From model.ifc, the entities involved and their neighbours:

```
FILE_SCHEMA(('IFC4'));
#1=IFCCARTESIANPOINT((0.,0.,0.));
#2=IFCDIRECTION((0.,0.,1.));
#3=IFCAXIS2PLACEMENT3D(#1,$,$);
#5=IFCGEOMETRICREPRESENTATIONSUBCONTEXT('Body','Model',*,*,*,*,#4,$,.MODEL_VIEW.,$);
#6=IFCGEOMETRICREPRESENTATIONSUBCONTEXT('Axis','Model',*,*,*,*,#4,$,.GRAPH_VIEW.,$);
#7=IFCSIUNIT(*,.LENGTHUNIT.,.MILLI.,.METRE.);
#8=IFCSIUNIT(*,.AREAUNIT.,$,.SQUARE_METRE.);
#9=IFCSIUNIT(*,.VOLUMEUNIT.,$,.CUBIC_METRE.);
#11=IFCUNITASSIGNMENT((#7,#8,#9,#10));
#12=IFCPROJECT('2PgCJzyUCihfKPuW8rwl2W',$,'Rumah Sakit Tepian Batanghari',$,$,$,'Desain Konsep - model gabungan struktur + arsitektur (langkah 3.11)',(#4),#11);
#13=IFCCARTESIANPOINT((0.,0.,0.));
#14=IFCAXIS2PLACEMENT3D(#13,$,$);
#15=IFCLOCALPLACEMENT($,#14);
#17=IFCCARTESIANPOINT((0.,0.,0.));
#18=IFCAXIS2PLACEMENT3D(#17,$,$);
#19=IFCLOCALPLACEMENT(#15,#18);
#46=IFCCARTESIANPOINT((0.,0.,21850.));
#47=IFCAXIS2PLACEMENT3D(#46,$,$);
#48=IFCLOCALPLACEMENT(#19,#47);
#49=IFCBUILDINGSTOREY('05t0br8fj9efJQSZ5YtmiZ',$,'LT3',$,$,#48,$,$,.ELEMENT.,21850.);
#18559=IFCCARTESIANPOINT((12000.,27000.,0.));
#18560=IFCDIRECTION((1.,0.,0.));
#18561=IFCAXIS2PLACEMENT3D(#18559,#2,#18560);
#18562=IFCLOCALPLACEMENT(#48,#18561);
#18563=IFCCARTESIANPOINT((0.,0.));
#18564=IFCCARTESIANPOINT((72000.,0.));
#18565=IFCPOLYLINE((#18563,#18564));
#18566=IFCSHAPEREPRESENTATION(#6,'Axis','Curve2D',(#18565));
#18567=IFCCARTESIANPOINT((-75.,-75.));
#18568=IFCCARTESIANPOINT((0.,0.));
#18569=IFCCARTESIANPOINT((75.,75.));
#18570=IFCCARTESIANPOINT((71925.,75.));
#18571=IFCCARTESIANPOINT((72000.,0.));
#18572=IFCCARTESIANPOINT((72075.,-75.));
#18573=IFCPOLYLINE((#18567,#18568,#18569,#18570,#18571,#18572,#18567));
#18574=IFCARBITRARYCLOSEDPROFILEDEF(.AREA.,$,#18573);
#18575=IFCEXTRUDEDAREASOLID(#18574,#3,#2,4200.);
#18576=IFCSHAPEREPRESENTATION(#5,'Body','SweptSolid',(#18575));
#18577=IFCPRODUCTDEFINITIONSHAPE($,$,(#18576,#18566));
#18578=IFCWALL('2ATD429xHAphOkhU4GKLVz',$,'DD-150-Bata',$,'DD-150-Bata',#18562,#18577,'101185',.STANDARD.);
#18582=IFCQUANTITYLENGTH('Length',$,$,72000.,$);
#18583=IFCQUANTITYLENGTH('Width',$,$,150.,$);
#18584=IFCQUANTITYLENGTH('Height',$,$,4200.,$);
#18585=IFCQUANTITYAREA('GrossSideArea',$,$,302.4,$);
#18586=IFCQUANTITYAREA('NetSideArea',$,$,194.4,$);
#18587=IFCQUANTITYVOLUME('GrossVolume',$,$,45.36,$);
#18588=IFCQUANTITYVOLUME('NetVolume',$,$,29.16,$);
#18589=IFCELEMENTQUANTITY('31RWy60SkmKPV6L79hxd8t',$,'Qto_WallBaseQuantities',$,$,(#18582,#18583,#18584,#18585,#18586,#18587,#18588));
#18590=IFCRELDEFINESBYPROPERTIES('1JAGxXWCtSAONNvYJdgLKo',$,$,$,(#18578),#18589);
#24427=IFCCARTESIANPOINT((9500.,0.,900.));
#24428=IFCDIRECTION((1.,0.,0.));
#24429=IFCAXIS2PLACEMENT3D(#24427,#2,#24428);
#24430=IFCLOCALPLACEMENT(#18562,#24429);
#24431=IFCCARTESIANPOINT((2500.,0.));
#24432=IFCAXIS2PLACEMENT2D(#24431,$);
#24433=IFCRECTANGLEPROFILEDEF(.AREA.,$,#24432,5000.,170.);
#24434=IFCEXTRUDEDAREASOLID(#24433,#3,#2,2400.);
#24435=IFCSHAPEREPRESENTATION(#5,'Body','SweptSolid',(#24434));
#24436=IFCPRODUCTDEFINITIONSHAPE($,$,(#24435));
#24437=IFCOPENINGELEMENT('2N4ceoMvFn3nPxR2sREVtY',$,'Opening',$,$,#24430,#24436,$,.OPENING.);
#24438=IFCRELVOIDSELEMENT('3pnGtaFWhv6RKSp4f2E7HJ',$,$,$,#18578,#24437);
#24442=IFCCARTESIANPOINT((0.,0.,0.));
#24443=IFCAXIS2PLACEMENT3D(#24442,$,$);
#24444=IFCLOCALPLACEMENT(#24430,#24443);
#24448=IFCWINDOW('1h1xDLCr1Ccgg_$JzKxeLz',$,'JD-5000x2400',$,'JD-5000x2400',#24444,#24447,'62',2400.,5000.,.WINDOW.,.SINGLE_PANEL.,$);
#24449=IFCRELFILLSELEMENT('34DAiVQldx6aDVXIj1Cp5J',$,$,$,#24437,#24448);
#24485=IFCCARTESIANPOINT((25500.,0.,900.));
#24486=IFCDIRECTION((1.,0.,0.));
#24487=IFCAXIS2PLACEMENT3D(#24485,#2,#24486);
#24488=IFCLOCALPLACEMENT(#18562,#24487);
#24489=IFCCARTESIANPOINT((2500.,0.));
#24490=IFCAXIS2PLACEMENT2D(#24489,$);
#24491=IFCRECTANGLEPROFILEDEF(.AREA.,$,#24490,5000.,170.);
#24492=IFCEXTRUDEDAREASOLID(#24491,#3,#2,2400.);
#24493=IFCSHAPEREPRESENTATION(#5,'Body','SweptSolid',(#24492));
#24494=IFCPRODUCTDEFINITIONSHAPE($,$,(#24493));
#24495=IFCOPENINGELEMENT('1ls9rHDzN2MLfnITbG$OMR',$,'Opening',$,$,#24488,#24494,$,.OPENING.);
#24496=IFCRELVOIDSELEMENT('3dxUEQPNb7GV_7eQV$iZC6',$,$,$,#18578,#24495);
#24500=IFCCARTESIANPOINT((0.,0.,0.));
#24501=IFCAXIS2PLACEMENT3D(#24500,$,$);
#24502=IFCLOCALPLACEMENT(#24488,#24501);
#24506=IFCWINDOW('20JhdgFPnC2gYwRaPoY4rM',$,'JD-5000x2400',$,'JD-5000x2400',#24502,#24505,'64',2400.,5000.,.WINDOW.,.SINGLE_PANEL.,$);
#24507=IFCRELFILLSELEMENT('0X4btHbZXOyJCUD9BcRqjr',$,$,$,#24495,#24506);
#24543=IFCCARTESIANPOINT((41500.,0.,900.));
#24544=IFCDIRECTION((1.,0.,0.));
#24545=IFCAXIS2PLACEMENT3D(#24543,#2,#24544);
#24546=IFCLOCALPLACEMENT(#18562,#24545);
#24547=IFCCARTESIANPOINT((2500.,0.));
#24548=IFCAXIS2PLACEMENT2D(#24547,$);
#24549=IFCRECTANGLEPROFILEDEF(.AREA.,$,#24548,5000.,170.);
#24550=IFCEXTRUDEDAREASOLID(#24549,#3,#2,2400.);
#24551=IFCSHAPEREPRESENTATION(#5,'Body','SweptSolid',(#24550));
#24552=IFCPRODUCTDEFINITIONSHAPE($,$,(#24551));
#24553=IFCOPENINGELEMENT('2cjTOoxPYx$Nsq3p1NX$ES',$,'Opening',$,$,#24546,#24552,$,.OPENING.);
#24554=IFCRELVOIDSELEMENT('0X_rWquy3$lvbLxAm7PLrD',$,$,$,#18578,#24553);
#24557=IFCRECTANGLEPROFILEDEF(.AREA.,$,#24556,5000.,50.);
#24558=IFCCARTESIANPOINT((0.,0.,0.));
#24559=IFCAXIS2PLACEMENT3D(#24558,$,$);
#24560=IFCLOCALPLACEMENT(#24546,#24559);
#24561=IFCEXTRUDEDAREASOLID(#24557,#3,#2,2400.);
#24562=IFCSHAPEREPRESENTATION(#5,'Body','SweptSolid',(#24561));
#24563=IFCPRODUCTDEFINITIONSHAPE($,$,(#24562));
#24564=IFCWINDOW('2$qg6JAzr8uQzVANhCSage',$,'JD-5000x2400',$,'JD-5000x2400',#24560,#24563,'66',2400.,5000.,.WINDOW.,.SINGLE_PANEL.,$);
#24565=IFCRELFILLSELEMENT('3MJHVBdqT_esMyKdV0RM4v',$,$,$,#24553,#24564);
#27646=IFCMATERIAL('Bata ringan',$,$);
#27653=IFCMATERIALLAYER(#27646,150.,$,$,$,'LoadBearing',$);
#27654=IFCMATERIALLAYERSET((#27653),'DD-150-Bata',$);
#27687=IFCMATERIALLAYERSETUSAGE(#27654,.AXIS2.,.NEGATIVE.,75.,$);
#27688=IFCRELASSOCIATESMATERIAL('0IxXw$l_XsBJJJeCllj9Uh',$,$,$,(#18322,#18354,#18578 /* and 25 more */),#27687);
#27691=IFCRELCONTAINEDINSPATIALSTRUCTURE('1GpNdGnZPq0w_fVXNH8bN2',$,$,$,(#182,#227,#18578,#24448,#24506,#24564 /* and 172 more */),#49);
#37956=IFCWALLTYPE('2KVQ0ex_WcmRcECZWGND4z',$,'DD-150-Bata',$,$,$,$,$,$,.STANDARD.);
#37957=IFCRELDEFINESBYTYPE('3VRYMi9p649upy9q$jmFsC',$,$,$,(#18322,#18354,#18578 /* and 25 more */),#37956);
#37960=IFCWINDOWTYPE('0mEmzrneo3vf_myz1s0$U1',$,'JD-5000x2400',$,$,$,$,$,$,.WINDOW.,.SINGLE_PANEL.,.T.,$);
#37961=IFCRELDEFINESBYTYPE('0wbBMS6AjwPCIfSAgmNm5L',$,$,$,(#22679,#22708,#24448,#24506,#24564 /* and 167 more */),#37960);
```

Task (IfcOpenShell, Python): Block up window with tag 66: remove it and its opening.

```python
import ifcopenshell
import ifcopenshell.api.feature
import ifcopenshell.api.pset
import ifcopenshell.api.root
import ifcopenshell.geom
import ifcopenshell.util.element
import ifcopenshell.util.shape
import ifcopenshell.util.unit

model = ifcopenshell.open("model.ifc")
area_scale = ifcopenshell.util.unit.calculate_unit_scale(model, "AREAUNIT")
volume_scale = ifcopenshell.util.unit.calculate_unit_scale(model, "VOLUMEUNIT")
settings = ifcopenshell.geom.settings()


def volume(element):
    """Net volume in cubic metres, openings subtracted."""
    shape = ifcopenshell.geom.create_shape(settings, element)
    return ifcopenshell.util.shape.get_volume(shape.geometry)


window = model.by_id(24564)
opening = window.FillsVoids[0].RelatingOpeningElement
wall = opening.VoidsElements[0].RelatingBuildingElement
before = volume(wall)

ifcopenshell.api.root.remove_product(model, product=window)
ifcopenshell.api.feature.remove_feature(model, feature=opening)

after = volume(wall)
thickness = 0.15  # wall thickness in metres

# Update the wall's stored quantities.
qto = model.by_id(ifcopenshell.util.element.get_pset(wall, "Qto_WallBaseQuantities", should_inherit=False)["id"])
ifcopenshell.api.pset.edit_qto(model, qto=qto, properties={
    "NetSideArea": after / thickness / area_scale,
    "NetVolume": after / volume_scale,
})

print(f"wall volume {before:.3f} -> {after:.3f} m3")

model.write("model_edited.ifc")
```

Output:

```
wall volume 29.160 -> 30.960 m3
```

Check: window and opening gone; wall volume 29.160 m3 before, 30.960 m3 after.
